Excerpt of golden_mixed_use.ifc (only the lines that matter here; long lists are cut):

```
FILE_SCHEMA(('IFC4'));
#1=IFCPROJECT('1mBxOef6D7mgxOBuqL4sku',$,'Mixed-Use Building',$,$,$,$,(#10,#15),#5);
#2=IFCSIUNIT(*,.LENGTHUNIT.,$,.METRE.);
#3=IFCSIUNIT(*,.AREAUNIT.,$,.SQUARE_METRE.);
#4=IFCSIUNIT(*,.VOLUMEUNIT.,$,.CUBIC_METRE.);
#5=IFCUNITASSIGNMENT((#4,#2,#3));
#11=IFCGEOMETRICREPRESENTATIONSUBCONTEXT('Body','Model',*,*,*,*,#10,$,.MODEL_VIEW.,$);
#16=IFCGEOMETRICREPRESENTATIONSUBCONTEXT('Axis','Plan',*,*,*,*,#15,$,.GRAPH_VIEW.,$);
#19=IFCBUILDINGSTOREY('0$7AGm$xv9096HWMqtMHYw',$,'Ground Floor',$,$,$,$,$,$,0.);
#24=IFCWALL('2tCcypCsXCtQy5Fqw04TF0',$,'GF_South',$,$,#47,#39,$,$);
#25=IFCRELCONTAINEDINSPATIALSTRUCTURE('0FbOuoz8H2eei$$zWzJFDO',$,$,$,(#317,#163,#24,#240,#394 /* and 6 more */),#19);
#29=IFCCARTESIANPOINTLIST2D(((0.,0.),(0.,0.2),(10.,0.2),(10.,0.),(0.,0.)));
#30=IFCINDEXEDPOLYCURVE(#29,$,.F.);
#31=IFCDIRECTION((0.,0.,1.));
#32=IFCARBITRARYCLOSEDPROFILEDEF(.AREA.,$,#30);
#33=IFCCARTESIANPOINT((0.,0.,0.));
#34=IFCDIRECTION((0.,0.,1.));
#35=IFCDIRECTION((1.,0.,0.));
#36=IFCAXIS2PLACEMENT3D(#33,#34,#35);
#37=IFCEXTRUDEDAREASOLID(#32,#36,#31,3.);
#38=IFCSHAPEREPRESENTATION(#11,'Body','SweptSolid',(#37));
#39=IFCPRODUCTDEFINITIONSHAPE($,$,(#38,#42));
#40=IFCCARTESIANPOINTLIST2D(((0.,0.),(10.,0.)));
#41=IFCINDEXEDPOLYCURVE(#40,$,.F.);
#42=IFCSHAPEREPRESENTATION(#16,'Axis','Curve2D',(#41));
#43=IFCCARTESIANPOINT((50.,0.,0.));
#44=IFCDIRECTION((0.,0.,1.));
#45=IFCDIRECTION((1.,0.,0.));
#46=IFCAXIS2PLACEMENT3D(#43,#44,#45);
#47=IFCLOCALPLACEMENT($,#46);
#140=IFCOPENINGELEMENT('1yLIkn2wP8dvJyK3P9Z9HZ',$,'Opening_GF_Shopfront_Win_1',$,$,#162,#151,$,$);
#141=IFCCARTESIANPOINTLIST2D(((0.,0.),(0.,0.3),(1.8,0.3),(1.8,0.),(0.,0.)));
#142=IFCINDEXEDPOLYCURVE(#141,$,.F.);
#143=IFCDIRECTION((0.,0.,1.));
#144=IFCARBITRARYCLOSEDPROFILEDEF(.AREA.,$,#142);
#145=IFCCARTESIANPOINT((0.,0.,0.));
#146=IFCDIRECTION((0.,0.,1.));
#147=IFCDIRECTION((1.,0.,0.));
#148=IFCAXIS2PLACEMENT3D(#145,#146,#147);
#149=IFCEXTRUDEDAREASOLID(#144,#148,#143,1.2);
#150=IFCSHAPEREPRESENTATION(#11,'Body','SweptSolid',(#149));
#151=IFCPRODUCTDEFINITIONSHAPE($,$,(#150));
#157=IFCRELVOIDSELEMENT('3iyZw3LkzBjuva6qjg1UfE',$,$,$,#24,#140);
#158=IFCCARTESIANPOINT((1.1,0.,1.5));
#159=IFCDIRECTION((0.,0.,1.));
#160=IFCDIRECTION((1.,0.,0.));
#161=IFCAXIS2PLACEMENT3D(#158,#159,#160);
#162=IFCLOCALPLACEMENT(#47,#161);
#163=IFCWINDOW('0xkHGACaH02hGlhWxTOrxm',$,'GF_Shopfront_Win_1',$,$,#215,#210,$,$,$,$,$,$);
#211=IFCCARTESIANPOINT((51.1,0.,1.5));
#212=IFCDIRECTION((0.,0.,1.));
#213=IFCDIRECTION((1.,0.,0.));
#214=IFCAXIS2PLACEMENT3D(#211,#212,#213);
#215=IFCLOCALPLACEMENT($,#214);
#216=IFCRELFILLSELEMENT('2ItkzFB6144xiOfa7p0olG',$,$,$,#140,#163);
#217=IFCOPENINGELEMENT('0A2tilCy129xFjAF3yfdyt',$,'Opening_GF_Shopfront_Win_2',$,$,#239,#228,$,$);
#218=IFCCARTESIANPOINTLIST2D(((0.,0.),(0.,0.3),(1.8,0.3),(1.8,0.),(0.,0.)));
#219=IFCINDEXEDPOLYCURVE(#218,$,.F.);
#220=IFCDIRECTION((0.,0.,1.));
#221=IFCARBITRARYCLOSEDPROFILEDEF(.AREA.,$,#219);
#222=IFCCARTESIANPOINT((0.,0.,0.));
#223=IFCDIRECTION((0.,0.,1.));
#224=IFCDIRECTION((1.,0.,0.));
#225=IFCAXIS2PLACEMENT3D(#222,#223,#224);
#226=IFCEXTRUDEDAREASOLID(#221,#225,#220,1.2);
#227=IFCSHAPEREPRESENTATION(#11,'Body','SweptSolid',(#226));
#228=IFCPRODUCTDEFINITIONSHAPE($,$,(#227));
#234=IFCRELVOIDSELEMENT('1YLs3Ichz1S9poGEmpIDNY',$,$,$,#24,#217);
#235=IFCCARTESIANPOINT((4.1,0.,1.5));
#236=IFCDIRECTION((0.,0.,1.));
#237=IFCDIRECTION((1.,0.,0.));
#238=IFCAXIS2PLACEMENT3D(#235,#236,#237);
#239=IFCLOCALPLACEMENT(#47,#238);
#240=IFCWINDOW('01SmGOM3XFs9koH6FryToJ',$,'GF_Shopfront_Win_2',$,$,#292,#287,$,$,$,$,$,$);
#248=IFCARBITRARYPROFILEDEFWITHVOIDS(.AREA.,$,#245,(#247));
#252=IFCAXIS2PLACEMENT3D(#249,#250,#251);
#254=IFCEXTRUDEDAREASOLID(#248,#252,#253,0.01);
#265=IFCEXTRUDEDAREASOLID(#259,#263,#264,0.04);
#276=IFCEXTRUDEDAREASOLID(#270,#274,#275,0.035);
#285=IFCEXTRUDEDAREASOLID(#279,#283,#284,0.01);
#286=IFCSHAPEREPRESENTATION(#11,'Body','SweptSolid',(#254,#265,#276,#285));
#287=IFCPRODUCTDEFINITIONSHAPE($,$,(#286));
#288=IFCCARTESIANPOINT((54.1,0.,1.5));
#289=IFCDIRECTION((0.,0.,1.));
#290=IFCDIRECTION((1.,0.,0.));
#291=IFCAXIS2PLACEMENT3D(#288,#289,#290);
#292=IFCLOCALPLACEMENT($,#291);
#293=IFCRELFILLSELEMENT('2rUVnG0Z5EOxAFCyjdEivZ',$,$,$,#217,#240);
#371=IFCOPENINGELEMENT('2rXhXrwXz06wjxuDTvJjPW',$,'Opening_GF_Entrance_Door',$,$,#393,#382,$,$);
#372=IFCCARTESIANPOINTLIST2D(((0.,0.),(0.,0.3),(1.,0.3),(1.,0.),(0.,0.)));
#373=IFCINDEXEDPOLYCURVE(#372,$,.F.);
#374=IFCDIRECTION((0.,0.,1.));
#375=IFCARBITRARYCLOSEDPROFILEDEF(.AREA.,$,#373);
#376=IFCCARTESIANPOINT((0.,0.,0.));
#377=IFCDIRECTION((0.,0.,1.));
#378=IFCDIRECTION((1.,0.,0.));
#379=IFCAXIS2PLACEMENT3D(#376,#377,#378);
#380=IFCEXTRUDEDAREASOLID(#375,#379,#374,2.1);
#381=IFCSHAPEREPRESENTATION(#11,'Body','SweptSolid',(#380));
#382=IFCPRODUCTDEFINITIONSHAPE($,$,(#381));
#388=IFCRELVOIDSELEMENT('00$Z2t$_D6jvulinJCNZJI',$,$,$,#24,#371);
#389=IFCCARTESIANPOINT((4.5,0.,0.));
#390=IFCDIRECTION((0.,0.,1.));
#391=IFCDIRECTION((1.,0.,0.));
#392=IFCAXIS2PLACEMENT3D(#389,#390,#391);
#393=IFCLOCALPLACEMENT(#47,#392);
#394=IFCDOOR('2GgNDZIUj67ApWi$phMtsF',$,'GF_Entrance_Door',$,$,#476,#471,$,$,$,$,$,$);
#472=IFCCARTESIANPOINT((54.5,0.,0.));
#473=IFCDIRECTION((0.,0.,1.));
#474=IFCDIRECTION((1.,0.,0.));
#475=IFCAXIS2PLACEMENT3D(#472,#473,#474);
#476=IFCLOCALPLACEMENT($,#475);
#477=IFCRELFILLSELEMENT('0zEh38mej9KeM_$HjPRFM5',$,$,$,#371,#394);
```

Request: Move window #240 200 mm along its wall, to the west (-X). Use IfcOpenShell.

```python
import ifcopenshell
import ifcopenshell.api.geometry
import ifcopenshell.util.placement

model = ifcopenshell.open("golden_mixed_use.ifc")

window = model.by_id(240)
opening = window.FillsVoids[0].RelatingOpeningElement
wall = opening.VoidsElements[0].RelatingBuildingElement

wall_matrix = ifcopenshell.util.placement.get_local_placement(wall.ObjectPlacement)
shift = wall_matrix[:3, 0] * -0.2
before = ifcopenshell.util.placement.get_local_placement(window.ObjectPlacement)[:3, 3].copy()

# The window is not placed relative to its opening, so move both.
for product in (opening, window):
    matrix = ifcopenshell.util.placement.get_local_placement(product.ObjectPlacement)
    matrix[:3, 3] += shift
    ifcopenshell.api.geometry.edit_object_placement(model, product=product, matrix=matrix, is_si=False)

after = ifcopenshell.util.placement.get_local_placement(window.ObjectPlacement)[:3, 3]
print("window moved by", (after - before).round(3) + 0.0)

model.write("golden_mixed_use_rev.ifc")
```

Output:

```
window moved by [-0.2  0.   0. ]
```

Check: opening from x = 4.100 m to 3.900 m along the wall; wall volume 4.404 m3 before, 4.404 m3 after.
